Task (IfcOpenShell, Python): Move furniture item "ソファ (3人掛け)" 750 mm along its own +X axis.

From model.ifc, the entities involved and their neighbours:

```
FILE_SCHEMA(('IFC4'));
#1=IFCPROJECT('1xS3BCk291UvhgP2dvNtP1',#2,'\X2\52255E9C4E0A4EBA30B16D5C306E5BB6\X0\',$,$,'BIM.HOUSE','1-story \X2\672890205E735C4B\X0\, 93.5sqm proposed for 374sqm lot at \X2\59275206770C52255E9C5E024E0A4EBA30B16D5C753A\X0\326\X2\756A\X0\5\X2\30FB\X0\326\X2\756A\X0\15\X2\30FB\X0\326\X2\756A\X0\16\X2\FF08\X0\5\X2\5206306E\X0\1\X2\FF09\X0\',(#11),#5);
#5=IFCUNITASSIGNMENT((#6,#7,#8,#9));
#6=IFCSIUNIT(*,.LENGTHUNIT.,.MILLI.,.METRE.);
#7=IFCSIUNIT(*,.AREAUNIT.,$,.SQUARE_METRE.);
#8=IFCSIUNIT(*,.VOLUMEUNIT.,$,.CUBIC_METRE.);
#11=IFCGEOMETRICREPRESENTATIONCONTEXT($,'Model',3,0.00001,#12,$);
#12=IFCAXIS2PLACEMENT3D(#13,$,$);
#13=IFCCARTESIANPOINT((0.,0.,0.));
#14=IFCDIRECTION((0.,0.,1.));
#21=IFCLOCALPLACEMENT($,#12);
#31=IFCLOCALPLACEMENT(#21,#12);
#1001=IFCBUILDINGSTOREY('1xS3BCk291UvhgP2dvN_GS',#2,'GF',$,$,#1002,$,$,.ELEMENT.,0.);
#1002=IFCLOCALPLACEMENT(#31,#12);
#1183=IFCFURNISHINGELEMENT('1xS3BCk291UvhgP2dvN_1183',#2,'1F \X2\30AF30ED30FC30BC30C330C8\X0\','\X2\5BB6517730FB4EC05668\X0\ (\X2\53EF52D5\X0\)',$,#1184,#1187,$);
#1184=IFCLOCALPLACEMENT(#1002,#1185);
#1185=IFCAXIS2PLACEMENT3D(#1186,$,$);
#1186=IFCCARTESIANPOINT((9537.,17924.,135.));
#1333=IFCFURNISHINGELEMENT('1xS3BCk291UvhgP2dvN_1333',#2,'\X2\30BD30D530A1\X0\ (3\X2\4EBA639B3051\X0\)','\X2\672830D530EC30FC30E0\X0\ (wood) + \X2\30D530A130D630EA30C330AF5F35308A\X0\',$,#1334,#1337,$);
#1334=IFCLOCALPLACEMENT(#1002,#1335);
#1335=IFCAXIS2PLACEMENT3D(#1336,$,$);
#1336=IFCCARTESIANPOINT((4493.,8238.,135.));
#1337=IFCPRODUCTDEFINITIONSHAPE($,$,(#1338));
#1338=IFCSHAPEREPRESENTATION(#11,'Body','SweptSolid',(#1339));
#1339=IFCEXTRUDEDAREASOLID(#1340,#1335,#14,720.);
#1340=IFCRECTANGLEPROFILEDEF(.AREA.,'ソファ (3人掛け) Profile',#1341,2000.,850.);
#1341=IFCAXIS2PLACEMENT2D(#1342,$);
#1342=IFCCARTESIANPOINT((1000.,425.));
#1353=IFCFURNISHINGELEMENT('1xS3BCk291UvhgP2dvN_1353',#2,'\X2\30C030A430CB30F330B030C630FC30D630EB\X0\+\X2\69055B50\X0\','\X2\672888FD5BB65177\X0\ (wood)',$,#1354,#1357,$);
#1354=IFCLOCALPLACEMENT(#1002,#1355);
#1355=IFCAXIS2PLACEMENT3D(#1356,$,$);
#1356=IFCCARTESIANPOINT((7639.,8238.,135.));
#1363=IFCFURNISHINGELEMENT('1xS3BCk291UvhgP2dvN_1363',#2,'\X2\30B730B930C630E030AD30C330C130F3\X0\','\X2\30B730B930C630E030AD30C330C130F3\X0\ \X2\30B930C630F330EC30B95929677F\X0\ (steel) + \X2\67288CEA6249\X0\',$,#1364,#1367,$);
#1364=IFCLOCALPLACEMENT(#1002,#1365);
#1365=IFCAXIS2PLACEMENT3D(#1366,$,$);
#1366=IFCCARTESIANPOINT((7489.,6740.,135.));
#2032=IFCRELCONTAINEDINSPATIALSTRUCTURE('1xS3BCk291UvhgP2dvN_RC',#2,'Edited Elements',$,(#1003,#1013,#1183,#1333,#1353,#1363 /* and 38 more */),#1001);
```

```python
import ifcopenshell
import ifcopenshell.api.geometry
import ifcopenshell.util.placement
import ifcopenshell.util.unit

model = ifcopenshell.open("model.ifc")
unit_scale = ifcopenshell.util.unit.calculate_unit_scale(model)

item = model.by_id(1333)
matrix = ifcopenshell.util.placement.get_local_placement(item.ObjectPlacement)
matrix[:3, 3] += matrix[:3, 0] * 0.75 / unit_scale
ifcopenshell.api.geometry.edit_object_placement(model, product=item, matrix=matrix, is_si=False)

print(ifcopenshell.util.placement.get_local_placement(item.ObjectPlacement).round(3) + 0.0)

model.write("model-out.ifc")
```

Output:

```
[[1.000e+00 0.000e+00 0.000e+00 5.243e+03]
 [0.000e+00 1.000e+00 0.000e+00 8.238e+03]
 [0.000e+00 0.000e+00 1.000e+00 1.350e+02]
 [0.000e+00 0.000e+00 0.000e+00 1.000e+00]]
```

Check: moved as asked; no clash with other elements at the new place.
